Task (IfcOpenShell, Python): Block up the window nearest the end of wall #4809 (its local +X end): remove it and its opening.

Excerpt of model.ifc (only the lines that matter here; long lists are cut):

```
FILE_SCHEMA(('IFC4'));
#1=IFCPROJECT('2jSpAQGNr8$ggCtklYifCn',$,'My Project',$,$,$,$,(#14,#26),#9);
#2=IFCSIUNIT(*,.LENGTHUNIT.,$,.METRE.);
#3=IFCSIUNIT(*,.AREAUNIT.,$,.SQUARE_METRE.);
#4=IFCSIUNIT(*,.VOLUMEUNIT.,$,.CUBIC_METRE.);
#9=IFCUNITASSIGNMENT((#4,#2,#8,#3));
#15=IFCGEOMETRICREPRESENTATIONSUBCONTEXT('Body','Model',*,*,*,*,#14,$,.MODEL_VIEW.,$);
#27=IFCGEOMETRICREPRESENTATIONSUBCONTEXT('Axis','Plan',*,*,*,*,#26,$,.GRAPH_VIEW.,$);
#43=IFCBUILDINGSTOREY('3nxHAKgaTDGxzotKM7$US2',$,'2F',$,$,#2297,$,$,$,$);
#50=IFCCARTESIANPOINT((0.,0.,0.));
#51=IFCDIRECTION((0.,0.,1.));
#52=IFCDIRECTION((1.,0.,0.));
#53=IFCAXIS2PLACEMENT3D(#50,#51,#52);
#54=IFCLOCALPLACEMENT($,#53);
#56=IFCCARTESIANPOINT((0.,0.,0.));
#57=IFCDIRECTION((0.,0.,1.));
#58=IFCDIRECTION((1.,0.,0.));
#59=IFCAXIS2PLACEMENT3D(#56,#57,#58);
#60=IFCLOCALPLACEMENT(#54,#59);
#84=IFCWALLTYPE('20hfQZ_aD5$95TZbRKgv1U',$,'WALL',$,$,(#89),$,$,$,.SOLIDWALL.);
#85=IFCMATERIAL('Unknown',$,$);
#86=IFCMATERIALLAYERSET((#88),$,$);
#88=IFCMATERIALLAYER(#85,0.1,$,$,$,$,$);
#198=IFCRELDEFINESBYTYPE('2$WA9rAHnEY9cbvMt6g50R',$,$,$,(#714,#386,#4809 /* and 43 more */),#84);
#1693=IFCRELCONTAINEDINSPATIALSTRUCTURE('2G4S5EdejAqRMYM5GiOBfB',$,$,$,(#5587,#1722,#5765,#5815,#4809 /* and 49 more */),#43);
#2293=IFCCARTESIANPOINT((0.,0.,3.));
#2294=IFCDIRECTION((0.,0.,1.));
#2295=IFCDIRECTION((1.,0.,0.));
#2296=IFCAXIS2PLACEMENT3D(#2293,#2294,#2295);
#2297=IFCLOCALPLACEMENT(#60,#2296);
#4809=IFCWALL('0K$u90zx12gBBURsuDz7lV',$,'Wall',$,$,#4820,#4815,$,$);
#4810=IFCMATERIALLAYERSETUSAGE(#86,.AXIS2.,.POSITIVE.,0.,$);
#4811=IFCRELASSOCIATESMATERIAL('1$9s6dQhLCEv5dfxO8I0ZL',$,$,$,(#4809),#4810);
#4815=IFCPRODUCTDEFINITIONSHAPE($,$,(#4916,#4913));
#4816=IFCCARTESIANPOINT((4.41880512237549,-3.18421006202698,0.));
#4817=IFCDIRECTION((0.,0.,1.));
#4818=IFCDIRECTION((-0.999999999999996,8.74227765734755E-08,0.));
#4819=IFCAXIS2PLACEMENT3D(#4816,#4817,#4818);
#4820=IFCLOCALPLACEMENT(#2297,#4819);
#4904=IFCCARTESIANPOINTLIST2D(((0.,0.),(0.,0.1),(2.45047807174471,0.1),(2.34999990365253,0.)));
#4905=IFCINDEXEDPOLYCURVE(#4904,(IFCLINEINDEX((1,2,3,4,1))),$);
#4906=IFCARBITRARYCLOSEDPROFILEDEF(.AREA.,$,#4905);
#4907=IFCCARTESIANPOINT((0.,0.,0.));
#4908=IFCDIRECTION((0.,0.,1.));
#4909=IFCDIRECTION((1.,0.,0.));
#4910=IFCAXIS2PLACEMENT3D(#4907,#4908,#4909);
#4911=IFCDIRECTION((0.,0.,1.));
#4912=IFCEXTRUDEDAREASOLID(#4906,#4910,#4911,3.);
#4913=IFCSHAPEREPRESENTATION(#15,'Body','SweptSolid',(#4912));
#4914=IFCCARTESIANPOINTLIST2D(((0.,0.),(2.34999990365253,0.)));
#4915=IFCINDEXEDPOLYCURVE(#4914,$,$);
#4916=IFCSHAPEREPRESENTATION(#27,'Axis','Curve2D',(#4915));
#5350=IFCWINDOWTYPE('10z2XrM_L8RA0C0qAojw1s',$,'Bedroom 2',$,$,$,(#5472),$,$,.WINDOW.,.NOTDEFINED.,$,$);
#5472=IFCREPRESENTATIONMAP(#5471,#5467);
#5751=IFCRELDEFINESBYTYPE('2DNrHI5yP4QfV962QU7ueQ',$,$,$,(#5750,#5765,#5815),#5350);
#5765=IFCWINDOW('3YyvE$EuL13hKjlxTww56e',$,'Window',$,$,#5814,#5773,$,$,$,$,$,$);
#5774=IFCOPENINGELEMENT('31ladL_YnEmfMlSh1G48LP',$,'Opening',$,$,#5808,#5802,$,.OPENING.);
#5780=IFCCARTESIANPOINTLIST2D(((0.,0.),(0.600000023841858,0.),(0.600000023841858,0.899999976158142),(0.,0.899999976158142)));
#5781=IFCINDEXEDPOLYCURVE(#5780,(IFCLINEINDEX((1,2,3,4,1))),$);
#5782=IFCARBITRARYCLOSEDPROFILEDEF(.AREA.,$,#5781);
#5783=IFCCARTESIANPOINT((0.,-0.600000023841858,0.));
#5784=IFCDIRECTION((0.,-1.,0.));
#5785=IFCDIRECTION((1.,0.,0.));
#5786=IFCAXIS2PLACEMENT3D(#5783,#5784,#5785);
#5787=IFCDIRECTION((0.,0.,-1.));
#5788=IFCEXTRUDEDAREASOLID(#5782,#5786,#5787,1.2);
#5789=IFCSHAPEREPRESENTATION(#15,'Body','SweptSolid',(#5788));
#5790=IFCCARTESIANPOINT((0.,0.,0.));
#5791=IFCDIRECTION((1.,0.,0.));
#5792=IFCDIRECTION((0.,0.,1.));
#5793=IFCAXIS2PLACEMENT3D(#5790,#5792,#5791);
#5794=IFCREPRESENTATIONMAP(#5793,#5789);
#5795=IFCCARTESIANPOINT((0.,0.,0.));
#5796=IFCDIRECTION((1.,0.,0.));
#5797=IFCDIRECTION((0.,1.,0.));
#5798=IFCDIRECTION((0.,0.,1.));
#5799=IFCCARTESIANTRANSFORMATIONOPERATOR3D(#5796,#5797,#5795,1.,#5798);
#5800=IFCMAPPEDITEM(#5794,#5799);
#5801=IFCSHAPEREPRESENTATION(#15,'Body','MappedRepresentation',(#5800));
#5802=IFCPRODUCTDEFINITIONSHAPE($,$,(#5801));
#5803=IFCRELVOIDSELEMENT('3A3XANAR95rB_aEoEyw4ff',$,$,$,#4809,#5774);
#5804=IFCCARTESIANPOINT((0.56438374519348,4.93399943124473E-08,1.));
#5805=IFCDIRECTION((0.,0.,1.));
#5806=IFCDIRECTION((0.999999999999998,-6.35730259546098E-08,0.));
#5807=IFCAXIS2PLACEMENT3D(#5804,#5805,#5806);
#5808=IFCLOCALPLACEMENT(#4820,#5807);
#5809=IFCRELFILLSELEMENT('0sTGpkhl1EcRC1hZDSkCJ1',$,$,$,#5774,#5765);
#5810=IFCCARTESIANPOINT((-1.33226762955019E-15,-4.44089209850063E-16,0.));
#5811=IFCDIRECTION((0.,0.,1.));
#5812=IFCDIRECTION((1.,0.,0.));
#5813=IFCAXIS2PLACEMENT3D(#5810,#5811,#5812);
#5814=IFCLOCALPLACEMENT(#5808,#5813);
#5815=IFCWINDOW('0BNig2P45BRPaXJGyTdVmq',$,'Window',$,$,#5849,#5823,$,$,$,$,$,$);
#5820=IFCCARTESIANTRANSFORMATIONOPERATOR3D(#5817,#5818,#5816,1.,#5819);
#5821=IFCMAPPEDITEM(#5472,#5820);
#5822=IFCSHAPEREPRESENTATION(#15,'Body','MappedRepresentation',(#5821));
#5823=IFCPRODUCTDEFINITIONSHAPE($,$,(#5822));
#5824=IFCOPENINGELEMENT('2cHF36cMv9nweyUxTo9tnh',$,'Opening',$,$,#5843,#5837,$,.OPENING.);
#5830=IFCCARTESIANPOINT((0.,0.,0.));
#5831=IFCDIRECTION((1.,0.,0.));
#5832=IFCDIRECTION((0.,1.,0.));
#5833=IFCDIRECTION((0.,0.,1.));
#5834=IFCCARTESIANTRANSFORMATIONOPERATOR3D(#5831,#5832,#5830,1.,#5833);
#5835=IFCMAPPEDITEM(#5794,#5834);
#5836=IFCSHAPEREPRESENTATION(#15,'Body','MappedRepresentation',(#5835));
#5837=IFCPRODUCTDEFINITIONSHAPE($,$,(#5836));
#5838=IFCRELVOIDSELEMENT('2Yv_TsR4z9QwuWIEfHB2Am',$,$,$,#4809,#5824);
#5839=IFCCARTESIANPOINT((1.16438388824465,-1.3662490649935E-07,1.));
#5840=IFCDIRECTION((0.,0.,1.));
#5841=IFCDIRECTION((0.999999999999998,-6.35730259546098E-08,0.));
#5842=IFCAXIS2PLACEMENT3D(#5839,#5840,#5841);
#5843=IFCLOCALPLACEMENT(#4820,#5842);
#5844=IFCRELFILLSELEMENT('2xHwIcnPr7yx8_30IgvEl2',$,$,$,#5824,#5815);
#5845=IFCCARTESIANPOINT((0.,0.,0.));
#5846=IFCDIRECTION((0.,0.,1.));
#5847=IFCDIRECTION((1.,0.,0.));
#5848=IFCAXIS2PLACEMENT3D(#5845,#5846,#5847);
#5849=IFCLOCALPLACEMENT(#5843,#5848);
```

```python
import ifcopenshell
import ifcopenshell.api.feature
import ifcopenshell.api.root
import ifcopenshell.geom
import ifcopenshell.util.shape

model = ifcopenshell.open("model.ifc")
settings = ifcopenshell.geom.settings()


def volume(element):
    """Net volume in cubic metres, openings subtracted."""
    shape = ifcopenshell.geom.create_shape(settings, element)
    return ifcopenshell.util.shape.get_volume(shape.geometry)


window = model.by_id(5815)
opening = window.FillsVoids[0].RelatingOpeningElement
wall = opening.VoidsElements[0].RelatingBuildingElement
before = volume(wall)

ifcopenshell.api.root.remove_product(model, product=window)
ifcopenshell.api.feature.remove_feature(model, feature=opening)

after = volume(wall)

print(f"wall volume {before:.3f} -> {after:.3f} m3")

model.write("model_edited.ifc")
```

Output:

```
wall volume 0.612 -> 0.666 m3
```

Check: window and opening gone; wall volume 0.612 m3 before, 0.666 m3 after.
